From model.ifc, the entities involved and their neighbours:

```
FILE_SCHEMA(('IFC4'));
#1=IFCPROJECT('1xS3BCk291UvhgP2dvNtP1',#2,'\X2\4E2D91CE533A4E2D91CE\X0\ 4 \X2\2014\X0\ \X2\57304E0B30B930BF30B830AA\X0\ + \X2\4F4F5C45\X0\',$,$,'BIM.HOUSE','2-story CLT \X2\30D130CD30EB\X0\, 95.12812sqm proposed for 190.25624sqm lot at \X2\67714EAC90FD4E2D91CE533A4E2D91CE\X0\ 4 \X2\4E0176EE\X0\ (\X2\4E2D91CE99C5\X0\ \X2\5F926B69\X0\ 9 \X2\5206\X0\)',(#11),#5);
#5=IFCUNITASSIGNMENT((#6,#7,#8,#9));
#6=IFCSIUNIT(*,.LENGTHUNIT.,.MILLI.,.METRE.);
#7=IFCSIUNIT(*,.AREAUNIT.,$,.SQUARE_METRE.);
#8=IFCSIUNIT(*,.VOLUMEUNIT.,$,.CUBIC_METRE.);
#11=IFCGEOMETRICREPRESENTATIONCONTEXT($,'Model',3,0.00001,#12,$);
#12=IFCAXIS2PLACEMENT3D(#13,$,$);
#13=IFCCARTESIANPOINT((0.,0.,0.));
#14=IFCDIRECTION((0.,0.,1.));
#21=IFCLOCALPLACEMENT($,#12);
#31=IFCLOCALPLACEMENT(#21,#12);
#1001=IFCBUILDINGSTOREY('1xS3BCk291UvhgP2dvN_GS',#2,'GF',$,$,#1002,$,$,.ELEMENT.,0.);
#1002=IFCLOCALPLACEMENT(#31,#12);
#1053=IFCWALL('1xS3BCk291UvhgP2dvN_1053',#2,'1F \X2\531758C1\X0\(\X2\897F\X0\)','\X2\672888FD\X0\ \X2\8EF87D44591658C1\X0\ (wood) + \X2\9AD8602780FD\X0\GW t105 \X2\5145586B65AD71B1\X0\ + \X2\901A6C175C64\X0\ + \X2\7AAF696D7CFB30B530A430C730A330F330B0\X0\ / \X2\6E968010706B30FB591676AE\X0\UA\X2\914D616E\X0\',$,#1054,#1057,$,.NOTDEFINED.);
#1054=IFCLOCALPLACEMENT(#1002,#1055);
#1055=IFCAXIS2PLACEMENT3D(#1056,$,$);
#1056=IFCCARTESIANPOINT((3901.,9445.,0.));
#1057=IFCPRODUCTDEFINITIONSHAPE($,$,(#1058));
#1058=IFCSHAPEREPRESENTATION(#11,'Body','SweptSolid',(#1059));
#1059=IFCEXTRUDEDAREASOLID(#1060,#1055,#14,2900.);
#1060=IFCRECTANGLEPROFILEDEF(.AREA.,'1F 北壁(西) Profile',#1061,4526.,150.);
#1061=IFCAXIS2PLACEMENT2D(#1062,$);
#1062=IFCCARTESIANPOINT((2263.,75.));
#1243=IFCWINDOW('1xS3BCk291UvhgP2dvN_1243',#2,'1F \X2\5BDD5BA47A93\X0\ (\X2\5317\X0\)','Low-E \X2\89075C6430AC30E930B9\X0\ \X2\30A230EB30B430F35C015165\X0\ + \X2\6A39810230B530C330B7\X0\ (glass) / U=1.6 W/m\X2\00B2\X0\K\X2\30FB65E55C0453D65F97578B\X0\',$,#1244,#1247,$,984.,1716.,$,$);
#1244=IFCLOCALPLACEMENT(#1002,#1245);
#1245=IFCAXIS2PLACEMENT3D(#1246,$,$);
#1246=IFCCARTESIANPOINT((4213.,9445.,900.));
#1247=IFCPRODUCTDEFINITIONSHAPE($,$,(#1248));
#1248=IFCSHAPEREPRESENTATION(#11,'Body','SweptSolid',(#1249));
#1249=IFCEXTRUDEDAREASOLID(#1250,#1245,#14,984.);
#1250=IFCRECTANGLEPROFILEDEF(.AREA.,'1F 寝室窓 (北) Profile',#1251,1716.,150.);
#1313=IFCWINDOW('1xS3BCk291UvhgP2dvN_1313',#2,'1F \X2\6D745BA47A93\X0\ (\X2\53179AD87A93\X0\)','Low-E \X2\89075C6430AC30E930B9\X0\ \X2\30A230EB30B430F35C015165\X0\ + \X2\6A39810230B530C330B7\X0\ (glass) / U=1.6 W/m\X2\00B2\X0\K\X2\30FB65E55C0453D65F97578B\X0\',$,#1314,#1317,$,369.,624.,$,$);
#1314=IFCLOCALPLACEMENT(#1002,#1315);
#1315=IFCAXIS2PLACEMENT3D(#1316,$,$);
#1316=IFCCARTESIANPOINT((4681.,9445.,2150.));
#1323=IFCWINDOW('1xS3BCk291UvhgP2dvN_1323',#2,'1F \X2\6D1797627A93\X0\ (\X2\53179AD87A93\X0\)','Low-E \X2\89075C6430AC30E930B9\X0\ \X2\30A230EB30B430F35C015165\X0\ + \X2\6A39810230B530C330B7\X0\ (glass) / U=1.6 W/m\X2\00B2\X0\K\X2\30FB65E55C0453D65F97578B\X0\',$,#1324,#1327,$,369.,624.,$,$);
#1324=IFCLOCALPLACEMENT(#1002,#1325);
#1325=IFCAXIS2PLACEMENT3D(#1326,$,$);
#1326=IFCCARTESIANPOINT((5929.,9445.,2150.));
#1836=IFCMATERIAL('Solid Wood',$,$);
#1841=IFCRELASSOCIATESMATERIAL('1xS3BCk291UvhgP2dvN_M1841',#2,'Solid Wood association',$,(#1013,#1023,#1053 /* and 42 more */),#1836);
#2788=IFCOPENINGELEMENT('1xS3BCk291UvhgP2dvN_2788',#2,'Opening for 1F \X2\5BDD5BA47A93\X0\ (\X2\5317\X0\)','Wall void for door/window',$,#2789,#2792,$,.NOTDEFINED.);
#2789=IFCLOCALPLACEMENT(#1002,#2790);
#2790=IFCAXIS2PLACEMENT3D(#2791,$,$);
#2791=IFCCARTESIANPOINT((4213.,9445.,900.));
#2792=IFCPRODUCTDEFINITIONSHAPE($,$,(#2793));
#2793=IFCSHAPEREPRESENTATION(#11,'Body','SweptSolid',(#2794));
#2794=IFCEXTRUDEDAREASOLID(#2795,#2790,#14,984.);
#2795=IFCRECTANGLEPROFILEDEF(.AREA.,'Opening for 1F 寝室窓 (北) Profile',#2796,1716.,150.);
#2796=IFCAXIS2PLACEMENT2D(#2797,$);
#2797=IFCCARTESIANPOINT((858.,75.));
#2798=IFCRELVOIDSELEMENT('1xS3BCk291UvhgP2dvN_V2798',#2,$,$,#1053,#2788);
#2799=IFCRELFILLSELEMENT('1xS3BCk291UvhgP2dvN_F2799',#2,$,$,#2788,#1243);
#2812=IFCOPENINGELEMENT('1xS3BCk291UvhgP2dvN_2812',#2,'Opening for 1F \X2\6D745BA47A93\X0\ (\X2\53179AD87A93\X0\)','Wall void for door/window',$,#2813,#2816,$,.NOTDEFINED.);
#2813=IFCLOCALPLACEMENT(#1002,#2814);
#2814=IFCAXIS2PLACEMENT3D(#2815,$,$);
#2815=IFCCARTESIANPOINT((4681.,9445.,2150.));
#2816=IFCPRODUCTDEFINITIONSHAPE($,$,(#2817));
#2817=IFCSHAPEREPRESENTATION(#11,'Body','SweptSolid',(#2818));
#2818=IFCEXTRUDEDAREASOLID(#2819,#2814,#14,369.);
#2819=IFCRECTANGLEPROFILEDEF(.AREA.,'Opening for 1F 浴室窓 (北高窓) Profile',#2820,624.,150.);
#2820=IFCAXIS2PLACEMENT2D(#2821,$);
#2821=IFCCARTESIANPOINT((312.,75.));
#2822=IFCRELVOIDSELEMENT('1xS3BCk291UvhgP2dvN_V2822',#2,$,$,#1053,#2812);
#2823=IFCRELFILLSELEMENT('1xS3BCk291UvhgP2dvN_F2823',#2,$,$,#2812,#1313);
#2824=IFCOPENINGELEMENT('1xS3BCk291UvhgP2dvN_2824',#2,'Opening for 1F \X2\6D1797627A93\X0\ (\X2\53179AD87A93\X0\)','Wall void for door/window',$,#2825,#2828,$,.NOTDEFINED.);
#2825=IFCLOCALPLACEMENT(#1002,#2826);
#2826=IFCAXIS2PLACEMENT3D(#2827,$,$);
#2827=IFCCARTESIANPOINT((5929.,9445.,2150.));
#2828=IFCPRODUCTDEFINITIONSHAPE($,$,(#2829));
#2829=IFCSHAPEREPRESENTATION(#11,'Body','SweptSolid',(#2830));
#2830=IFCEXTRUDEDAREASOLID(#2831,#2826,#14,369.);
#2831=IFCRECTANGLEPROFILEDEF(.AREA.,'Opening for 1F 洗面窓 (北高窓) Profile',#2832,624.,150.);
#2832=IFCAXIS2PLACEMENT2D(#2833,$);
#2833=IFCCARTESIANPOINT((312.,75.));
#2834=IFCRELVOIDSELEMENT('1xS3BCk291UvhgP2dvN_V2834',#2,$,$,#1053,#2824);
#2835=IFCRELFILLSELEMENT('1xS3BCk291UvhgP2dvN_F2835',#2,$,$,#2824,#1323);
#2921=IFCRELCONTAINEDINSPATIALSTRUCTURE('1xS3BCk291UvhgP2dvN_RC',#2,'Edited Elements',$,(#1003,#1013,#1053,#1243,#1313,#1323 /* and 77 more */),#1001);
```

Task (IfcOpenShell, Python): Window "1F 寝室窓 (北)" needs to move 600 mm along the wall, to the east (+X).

```python
import ifcopenshell
import ifcopenshell.api.geometry
import ifcopenshell.util.placement
import ifcopenshell.util.unit

model = ifcopenshell.open("model.ifc")
unit_scale = ifcopenshell.util.unit.calculate_unit_scale(model)

window = model.by_guid("1xS3BCk291UvhgP2dvN_1243")
opening = window.FillsVoids[0].RelatingOpeningElement
wall = opening.VoidsElements[0].RelatingBuildingElement

wall_matrix = ifcopenshell.util.placement.get_local_placement(wall.ObjectPlacement)
shift = wall_matrix[:3, 0] * 0.6 / unit_scale
before = ifcopenshell.util.placement.get_local_placement(window.ObjectPlacement)[:3, 3].copy()

# The window is not placed relative to its opening, so move both.
for product in (opening, window):
    matrix = ifcopenshell.util.placement.get_local_placement(product.ObjectPlacement)
    matrix[:3, 3] += shift
    ifcopenshell.api.geometry.edit_object_placement(model, product=product, matrix=matrix, is_si=False)

after = ifcopenshell.util.placement.get_local_placement(window.ObjectPlacement)[:3, 3]
print("window moved by", (after - before).round(3) + 0.0)

model.write("model_rev.ifc")
```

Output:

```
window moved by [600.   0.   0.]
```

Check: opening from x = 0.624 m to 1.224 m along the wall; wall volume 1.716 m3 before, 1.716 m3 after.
